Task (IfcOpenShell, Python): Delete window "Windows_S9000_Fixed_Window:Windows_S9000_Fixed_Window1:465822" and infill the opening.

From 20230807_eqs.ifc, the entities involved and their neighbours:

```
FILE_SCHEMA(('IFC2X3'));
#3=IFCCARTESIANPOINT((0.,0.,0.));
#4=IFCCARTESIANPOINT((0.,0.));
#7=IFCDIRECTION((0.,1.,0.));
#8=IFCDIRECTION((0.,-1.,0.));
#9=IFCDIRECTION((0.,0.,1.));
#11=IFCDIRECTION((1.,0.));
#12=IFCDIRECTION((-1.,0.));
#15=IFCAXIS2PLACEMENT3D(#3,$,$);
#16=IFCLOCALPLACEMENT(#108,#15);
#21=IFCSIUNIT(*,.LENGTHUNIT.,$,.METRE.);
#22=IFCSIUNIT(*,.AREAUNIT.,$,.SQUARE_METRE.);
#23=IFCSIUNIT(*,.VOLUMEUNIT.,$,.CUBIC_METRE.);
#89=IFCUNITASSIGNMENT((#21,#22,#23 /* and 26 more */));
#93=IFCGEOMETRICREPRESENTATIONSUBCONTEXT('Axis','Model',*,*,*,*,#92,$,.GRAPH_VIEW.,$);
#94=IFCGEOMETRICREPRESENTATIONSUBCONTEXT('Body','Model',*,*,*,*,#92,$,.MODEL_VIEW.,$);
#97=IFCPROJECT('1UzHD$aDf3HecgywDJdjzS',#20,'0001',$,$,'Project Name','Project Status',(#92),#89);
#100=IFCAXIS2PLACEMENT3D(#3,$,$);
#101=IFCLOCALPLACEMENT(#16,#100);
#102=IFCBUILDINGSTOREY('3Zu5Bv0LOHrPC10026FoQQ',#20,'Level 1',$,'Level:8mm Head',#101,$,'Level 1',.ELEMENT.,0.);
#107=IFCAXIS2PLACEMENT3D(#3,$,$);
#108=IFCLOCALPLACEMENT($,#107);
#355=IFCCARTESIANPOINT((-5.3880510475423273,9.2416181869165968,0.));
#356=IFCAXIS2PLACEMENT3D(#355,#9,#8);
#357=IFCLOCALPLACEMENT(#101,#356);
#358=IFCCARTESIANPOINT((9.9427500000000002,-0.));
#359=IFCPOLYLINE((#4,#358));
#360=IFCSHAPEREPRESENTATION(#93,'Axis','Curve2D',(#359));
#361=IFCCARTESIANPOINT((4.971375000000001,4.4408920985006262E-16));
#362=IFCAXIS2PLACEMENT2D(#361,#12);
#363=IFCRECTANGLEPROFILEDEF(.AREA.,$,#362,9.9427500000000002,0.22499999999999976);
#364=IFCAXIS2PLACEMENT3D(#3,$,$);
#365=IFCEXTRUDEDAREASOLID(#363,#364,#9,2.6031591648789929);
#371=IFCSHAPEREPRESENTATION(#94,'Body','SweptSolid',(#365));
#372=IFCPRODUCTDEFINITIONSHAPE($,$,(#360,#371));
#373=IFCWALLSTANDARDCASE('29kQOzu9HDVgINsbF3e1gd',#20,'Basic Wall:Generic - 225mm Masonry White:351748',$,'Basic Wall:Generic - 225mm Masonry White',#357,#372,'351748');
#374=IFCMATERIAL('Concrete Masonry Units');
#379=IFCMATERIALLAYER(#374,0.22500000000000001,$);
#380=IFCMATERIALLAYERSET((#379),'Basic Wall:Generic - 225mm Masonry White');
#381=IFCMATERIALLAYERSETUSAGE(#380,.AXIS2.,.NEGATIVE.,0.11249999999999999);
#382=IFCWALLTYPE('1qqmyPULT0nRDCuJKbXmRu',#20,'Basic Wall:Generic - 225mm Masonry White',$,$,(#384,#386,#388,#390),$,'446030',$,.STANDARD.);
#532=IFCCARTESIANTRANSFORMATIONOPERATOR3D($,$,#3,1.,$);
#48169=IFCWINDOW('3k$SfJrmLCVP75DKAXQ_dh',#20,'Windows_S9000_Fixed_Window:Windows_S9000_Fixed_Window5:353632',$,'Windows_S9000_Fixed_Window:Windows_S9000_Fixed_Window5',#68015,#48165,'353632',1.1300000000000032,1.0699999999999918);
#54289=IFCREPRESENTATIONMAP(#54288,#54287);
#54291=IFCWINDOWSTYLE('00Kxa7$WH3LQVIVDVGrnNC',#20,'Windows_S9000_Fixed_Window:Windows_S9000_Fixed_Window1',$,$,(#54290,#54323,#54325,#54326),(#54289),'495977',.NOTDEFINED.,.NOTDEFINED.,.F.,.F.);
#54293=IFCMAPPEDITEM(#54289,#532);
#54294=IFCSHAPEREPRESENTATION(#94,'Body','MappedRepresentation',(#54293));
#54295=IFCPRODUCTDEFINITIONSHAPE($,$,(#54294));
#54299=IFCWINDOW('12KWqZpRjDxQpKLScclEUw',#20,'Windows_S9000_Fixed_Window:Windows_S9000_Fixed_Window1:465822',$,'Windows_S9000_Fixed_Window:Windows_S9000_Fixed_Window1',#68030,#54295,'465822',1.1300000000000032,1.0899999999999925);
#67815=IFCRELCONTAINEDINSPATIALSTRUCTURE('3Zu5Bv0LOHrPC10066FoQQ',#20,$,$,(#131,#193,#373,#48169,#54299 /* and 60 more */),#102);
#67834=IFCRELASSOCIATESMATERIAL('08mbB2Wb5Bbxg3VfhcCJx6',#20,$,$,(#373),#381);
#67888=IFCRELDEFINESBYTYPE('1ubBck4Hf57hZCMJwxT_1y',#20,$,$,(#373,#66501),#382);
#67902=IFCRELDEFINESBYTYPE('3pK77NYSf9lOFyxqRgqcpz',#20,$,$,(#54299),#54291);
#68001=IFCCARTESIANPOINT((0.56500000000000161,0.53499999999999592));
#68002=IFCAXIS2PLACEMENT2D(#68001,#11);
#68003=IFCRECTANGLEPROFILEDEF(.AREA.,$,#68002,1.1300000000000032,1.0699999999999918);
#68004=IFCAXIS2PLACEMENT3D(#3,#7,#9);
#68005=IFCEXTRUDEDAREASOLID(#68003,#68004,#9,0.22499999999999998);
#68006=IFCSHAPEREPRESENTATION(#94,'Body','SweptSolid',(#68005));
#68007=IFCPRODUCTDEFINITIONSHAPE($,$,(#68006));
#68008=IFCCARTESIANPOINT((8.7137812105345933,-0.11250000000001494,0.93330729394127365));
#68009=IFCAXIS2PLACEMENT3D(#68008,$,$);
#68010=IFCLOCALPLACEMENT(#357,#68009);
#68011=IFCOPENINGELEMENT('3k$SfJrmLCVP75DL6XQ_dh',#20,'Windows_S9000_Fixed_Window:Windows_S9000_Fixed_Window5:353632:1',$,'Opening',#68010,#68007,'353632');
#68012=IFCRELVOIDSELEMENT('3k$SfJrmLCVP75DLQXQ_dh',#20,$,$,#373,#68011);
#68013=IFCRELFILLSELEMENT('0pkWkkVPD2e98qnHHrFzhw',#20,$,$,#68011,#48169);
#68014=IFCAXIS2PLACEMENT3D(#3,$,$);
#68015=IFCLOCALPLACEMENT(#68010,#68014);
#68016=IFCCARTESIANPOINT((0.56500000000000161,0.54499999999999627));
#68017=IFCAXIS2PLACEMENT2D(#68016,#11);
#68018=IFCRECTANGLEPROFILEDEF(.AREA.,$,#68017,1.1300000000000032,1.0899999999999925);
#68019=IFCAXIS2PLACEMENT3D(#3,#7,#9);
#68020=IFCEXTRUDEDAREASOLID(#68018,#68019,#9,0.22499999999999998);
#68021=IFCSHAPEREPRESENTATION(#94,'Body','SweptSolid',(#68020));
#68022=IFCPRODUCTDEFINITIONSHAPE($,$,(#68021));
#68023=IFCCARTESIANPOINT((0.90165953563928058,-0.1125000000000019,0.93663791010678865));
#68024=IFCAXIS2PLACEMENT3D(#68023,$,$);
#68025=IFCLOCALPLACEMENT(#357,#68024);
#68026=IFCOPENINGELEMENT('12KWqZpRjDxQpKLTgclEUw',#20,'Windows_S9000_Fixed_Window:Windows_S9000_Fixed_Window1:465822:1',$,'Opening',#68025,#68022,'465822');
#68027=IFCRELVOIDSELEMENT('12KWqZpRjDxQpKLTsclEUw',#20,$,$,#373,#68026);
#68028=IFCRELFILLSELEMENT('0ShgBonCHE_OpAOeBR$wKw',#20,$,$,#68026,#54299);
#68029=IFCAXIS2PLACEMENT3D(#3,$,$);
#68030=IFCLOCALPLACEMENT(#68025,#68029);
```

```python
import ifcopenshell
import ifcopenshell.api.feature
import ifcopenshell.api.root
import ifcopenshell.geom
import ifcopenshell.util.shape

model = ifcopenshell.open("20230807_eqs.ifc")
settings = ifcopenshell.geom.settings()


def volume(element):
    """Net volume in cubic metres, openings subtracted."""
    shape = ifcopenshell.geom.create_shape(settings, element)
    return ifcopenshell.util.shape.get_volume(shape.geometry)


window = model.by_guid("12KWqZpRjDxQpKLScclEUw")
opening = window.FillsVoids[0].RelatingOpeningElement
wall = opening.VoidsElements[0].RelatingBuildingElement
before = volume(wall)

ifcopenshell.api.root.remove_product(model, product=window)
ifcopenshell.api.feature.remove_feature(model, feature=opening)

after = volume(wall)

print(f"wall volume {before:.3f} -> {after:.3f} m3")

model.write("20230807_eqs_v2.ifc")
```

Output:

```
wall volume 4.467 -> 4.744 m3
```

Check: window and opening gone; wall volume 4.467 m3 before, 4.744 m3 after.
